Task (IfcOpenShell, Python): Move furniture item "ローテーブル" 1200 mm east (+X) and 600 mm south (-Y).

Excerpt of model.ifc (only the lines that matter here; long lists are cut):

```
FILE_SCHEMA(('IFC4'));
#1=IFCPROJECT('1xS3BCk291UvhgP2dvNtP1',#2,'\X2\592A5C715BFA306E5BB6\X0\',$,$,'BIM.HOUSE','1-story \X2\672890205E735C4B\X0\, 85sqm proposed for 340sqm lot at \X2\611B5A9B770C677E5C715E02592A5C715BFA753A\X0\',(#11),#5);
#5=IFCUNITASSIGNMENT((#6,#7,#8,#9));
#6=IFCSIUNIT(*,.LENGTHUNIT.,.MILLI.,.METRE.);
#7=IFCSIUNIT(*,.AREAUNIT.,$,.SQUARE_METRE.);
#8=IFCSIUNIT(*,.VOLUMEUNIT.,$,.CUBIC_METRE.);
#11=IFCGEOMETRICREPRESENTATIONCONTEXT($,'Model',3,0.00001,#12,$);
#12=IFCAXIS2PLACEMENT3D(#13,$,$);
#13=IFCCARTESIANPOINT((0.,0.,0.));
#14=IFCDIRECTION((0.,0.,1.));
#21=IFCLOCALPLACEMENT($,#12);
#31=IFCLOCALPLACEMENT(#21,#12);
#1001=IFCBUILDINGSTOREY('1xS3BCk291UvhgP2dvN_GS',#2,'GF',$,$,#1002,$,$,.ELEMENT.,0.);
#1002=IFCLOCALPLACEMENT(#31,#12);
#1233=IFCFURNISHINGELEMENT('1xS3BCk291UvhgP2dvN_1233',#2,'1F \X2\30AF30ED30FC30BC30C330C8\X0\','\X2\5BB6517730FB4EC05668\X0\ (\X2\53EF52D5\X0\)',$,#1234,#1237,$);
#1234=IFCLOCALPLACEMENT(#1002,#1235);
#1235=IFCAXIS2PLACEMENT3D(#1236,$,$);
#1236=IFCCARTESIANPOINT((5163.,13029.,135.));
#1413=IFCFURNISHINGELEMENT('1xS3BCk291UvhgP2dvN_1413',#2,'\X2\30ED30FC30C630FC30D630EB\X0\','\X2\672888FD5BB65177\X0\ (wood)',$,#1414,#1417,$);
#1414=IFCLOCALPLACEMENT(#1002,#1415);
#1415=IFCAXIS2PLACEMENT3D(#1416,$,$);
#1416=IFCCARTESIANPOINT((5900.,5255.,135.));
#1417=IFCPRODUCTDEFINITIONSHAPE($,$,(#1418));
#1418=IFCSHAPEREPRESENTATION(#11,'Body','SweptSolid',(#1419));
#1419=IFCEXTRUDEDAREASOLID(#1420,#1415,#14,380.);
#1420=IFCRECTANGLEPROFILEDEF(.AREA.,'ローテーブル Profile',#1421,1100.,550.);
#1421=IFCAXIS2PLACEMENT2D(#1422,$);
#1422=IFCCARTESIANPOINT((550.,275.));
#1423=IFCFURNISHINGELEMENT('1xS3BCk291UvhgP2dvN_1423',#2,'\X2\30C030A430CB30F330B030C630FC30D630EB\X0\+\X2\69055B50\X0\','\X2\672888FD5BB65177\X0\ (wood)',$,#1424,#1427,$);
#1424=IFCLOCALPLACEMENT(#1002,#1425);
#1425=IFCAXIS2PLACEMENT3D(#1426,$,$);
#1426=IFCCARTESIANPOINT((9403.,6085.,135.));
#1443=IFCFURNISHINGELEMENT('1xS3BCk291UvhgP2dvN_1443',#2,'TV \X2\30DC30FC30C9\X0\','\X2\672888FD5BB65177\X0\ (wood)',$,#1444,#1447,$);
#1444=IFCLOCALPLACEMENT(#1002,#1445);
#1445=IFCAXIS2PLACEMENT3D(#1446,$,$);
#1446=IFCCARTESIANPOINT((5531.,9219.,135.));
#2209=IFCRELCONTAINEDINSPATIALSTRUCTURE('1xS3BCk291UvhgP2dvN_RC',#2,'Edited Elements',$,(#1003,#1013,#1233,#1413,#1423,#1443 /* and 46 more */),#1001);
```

```python
import ifcopenshell
import ifcopenshell.api.geometry
import ifcopenshell.util.placement

model = ifcopenshell.open("model.ifc")

item = model.by_guid("1xS3BCk291UvhgP2dvN_1413")
matrix = ifcopenshell.util.placement.get_local_placement(item.ObjectPlacement)
matrix[0, 3] += 1200.0
matrix[1, 3] -= 600.0
ifcopenshell.api.geometry.edit_object_placement(model, product=item, matrix=matrix, is_si=False)

print(ifcopenshell.util.placement.get_local_placement(item.ObjectPlacement).round(3) + 0.0)

model.write("model_updated.ifc")
```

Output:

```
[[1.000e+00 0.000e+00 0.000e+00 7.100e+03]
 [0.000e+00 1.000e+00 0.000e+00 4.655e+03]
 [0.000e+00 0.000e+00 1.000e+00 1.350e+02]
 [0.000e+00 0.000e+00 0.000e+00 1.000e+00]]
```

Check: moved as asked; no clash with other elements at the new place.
